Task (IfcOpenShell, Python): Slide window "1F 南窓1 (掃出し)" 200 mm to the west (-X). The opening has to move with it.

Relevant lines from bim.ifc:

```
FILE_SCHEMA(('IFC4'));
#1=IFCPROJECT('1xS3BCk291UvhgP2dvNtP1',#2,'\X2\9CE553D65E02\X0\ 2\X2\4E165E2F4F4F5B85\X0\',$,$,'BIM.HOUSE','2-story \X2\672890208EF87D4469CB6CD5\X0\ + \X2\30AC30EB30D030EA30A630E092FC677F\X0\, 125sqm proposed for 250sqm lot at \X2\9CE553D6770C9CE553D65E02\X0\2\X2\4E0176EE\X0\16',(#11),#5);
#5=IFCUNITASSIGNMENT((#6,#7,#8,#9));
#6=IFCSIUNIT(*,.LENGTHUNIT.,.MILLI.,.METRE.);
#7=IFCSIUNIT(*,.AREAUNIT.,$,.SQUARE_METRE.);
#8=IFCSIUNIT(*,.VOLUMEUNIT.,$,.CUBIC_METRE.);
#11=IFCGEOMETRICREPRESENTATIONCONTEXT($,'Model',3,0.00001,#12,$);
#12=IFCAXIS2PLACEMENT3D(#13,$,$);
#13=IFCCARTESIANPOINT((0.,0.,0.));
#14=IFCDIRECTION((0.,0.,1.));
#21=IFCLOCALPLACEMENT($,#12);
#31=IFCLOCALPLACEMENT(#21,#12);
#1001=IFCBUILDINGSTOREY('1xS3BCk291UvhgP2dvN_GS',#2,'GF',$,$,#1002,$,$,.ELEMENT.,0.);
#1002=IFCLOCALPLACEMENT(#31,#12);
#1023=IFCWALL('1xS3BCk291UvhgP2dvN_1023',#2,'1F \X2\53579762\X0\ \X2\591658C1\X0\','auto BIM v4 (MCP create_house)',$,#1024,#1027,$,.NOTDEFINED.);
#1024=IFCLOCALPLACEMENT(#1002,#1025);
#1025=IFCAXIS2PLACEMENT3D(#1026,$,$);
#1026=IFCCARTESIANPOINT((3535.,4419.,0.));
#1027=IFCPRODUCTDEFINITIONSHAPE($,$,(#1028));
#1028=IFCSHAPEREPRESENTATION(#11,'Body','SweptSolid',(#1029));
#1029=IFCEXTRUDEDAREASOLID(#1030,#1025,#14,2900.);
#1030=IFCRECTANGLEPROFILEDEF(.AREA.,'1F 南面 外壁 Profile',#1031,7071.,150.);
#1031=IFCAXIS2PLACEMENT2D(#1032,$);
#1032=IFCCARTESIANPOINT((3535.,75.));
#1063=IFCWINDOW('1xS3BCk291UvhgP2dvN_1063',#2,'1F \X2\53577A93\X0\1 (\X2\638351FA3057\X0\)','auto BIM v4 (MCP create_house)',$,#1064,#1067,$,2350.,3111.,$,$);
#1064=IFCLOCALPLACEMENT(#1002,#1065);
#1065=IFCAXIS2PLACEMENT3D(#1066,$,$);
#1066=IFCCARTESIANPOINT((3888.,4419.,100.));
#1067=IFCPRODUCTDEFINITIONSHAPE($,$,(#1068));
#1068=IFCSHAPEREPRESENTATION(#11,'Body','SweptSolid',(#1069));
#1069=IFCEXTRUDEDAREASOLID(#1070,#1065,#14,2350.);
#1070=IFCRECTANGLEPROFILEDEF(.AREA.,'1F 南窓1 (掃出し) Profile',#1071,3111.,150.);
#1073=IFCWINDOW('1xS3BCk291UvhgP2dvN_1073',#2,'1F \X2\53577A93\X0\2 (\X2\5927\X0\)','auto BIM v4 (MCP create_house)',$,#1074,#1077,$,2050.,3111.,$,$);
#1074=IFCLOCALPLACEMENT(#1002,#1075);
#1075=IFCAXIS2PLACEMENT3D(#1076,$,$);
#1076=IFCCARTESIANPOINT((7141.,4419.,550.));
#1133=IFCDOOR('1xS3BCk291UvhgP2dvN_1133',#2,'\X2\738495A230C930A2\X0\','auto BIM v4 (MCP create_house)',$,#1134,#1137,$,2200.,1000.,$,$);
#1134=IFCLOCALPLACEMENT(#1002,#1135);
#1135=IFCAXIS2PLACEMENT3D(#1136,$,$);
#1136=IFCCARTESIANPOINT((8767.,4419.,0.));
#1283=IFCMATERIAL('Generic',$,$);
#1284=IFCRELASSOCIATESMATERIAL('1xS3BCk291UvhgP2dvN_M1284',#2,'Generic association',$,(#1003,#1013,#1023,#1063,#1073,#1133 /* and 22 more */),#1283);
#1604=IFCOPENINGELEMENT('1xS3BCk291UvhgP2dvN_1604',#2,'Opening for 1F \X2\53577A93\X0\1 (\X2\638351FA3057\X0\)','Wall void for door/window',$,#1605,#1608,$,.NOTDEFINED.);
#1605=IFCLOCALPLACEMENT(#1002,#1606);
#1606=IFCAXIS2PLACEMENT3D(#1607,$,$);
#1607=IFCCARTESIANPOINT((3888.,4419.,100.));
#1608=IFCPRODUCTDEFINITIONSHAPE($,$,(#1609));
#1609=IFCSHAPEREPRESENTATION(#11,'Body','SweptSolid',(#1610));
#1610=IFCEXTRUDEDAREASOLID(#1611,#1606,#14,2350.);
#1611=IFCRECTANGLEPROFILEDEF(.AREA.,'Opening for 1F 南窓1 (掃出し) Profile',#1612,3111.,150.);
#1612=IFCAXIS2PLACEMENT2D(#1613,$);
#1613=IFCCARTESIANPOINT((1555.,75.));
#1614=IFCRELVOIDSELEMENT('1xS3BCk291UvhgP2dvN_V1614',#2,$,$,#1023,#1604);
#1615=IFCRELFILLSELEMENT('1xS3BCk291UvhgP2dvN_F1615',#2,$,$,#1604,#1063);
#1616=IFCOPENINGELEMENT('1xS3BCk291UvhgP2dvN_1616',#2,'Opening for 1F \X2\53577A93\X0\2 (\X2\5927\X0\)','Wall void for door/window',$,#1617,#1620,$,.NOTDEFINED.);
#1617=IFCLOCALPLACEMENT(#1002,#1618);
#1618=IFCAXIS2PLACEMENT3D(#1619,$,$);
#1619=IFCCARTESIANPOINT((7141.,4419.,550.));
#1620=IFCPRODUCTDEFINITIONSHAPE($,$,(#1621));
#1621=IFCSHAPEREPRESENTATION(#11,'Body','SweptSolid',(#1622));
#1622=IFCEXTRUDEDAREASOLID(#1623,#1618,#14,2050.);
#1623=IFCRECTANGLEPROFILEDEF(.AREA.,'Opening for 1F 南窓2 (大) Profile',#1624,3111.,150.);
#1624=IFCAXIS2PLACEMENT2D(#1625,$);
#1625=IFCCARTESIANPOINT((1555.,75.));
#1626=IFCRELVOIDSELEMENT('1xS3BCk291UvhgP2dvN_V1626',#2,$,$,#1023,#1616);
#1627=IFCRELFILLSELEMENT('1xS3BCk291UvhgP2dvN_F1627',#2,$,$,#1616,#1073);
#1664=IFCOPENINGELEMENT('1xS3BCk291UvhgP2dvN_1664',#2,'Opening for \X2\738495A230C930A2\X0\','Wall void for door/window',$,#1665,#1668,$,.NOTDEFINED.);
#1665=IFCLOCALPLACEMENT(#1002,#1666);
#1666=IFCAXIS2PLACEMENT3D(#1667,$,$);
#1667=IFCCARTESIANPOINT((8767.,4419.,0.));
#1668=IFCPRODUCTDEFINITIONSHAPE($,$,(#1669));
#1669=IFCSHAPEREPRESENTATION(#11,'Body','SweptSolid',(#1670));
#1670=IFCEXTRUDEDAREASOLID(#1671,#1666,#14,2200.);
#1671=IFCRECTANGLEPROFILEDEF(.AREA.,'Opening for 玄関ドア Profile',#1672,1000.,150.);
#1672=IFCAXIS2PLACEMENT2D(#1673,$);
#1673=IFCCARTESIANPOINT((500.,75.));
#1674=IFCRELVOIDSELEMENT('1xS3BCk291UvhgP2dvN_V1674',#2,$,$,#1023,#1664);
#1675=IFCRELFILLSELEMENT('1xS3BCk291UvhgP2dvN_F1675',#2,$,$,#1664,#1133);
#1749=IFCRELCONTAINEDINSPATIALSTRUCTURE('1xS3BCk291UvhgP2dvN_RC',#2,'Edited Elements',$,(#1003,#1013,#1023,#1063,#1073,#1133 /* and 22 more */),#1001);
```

```python
import ifcopenshell
import ifcopenshell.api.geometry
import ifcopenshell.util.placement
import ifcopenshell.util.unit

model = ifcopenshell.open("bim.ifc")
unit_scale = ifcopenshell.util.unit.calculate_unit_scale(model)

window = model.by_guid("1xS3BCk291UvhgP2dvN_1063")
opening = window.FillsVoids[0].RelatingOpeningElement
wall = opening.VoidsElements[0].RelatingBuildingElement

wall_matrix = ifcopenshell.util.placement.get_local_placement(wall.ObjectPlacement)
shift = wall_matrix[:3, 0] * -0.2 / unit_scale
before = ifcopenshell.util.placement.get_local_placement(window.ObjectPlacement)[:3, 3].copy()

# The window is not placed relative to its opening, so move both.
for product in (opening, window):
    matrix = ifcopenshell.util.placement.get_local_placement(product.ObjectPlacement)
    matrix[:3, 3] += shift
    ifcopenshell.api.geometry.edit_object_placement(model, product=product, matrix=matrix, is_si=False)

after = ifcopenshell.util.placement.get_local_placement(window.ObjectPlacement)[:3, 3]
print("window moved by", (after - before).round(3) + 0.0)

model.write("bim-out.ifc")
```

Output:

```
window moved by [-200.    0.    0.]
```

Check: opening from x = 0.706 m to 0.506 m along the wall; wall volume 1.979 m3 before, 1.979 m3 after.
